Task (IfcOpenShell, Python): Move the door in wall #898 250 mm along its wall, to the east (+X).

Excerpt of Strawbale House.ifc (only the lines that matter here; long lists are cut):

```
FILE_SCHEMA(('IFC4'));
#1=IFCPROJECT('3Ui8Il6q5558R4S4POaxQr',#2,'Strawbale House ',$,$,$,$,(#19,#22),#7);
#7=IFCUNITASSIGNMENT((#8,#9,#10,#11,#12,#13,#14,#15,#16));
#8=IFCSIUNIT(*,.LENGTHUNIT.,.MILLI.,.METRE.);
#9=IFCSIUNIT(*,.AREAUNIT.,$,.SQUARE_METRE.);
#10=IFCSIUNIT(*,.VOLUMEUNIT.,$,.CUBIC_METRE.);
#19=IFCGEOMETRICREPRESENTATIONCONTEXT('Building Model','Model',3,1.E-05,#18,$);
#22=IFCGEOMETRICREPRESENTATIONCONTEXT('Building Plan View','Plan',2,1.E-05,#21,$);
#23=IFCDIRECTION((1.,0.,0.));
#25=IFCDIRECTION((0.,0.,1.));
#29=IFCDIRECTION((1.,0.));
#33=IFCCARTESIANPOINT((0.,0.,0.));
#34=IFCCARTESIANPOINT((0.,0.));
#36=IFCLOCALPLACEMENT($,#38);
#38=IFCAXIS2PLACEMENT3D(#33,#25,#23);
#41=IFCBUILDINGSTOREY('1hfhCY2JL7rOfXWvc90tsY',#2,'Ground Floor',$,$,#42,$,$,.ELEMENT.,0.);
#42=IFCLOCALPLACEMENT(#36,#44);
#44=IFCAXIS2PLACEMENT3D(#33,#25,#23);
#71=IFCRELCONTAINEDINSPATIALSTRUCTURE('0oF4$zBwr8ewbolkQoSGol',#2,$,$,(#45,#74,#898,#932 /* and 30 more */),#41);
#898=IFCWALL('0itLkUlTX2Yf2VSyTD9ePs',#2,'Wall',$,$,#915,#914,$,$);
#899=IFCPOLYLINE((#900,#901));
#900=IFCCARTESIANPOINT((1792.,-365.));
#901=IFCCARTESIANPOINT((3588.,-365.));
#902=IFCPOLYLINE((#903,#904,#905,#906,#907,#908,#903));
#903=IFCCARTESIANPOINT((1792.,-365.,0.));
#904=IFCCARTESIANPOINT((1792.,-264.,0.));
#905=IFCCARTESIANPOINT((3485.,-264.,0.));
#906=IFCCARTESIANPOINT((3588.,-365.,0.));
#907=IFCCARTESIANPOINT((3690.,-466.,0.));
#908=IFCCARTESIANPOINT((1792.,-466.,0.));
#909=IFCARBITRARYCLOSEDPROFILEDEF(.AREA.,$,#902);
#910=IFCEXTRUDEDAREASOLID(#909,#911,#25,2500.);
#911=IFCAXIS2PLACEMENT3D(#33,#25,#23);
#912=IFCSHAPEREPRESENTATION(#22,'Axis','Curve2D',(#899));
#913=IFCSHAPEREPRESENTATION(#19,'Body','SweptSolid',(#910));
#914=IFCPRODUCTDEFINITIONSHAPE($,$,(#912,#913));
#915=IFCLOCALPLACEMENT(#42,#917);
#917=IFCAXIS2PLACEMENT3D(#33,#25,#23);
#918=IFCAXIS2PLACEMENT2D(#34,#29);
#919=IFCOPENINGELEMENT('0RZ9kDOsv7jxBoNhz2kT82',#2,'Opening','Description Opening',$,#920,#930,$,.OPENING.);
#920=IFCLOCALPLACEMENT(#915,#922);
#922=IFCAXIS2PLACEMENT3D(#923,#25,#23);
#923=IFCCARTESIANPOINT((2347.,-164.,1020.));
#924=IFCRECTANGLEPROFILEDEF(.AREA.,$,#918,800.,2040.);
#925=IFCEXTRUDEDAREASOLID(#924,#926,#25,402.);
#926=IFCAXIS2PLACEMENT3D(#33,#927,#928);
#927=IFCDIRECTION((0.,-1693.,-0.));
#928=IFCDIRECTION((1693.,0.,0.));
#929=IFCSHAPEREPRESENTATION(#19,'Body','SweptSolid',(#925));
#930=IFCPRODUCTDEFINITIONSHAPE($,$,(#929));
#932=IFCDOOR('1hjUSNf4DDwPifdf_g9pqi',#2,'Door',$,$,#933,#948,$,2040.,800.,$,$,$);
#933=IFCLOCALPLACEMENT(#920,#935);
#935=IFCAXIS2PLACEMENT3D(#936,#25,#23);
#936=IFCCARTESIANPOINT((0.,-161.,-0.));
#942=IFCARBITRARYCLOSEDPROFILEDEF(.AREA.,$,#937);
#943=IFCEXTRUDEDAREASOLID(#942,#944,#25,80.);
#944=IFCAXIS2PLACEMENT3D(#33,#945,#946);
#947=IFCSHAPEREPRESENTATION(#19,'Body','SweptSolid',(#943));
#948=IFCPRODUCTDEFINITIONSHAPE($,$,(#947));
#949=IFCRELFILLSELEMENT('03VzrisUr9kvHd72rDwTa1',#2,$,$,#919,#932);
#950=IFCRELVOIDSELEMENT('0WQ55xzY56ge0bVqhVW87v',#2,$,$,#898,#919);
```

```python
import ifcopenshell
import ifcopenshell.api.geometry
import ifcopenshell.util.placement
import ifcopenshell.util.unit

model = ifcopenshell.open("Strawbale House.ifc")
unit_scale = ifcopenshell.util.unit.calculate_unit_scale(model)

door = model.by_id(932)
opening = door.FillsVoids[0].RelatingOpeningElement
wall = opening.VoidsElements[0].RelatingBuildingElement

wall_matrix = ifcopenshell.util.placement.get_local_placement(wall.ObjectPlacement)
shift = wall_matrix[:3, 0] * 0.25 / unit_scale
before = ifcopenshell.util.placement.get_local_placement(door.ObjectPlacement)[:3, 3].copy()

# The door is placed relative to its opening, so it follows when the opening moves.
matrix = ifcopenshell.util.placement.get_local_placement(opening.ObjectPlacement)
matrix[:3, 3] += shift
ifcopenshell.api.geometry.edit_object_placement(
    model, product=opening, matrix=matrix, is_si=False, should_transform_children=True
)

after = ifcopenshell.util.placement.get_local_placement(door.ObjectPlacement)[:3, 3]
print("door moved by", (after - before).round(3) + 0.0)

model.write("Strawbale House_updated.ifc")
```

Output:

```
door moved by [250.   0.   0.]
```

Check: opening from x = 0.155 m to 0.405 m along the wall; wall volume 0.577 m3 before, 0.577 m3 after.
